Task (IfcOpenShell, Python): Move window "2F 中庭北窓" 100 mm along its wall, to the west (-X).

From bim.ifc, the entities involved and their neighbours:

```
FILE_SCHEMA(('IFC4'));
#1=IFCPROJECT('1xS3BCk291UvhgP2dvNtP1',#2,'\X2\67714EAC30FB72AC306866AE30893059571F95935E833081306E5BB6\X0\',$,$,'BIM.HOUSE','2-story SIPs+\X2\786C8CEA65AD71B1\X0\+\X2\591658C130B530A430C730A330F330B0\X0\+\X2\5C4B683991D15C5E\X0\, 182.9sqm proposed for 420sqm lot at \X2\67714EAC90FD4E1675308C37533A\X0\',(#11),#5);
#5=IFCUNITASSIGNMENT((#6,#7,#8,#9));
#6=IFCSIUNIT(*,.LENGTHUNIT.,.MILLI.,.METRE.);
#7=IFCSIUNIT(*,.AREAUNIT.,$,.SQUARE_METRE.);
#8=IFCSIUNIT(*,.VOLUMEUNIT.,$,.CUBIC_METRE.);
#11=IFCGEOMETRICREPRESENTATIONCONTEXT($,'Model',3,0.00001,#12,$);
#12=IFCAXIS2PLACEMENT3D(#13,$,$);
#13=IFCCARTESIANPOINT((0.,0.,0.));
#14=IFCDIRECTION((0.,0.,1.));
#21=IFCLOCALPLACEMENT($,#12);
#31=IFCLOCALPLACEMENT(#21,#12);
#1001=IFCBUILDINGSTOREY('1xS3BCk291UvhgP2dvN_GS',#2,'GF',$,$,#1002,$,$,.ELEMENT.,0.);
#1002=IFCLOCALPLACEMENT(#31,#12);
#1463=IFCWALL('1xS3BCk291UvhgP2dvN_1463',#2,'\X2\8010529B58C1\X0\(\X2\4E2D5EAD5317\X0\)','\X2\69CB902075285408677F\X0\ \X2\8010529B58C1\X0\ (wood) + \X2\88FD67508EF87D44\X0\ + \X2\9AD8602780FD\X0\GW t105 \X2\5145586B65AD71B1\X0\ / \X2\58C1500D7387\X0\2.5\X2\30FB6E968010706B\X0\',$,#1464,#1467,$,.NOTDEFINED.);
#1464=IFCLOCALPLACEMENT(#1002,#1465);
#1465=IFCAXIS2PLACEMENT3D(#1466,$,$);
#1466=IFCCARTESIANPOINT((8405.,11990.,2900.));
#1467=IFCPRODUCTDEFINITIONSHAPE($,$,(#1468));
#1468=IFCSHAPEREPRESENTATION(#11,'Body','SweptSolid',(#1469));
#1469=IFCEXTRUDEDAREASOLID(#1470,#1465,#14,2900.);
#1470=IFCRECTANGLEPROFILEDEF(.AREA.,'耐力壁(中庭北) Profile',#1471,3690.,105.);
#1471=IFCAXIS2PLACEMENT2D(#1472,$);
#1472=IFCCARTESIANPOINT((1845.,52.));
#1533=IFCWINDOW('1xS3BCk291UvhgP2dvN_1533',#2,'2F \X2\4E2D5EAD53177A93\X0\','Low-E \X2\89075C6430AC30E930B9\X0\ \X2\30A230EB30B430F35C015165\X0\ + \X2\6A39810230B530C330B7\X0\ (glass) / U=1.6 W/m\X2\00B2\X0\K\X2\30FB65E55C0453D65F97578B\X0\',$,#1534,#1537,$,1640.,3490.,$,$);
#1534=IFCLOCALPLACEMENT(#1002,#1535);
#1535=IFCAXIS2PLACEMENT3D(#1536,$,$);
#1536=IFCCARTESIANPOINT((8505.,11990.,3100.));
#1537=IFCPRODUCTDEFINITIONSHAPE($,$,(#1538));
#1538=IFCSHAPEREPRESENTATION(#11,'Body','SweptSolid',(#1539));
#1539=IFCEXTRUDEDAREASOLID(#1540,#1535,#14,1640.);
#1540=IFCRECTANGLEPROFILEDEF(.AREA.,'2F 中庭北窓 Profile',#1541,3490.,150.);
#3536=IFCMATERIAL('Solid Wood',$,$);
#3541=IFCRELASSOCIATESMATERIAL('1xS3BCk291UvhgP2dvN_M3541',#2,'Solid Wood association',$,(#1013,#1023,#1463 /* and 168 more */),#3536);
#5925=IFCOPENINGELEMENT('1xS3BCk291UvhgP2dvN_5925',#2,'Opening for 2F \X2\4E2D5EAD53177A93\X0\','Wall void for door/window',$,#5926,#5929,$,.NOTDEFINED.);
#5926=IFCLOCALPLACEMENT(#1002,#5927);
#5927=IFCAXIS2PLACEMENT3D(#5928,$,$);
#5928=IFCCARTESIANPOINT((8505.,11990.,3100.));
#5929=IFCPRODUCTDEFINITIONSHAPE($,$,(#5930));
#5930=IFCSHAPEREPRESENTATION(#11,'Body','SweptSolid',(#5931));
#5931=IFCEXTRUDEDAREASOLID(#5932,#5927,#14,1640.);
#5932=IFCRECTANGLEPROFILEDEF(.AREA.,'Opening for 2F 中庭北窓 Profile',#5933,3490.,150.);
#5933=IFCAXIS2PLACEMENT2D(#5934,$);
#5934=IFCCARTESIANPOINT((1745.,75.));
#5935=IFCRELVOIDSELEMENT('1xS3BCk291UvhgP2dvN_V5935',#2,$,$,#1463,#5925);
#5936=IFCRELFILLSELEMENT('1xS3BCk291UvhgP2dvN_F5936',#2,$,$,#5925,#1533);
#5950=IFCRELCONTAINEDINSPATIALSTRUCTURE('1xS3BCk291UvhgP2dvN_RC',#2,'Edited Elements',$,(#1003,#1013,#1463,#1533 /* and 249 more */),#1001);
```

```python
import ifcopenshell
import ifcopenshell.api.geometry
import ifcopenshell.util.placement
import ifcopenshell.util.unit

model = ifcopenshell.open("bim.ifc")
unit_scale = ifcopenshell.util.unit.calculate_unit_scale(model)

window = model.by_id(1533)
opening = window.FillsVoids[0].RelatingOpeningElement
wall = opening.VoidsElements[0].RelatingBuildingElement

wall_matrix = ifcopenshell.util.placement.get_local_placement(wall.ObjectPlacement)
shift = wall_matrix[:3, 0] * -0.1 / unit_scale
before = ifcopenshell.util.placement.get_local_placement(window.ObjectPlacement)[:3, 3].copy()

# The window is not placed relative to its opening, so move both.
for product in (opening, window):
    matrix = ifcopenshell.util.placement.get_local_placement(product.ObjectPlacement)
    matrix[:3, 3] += shift
    ifcopenshell.api.geometry.edit_object_placement(model, product=product, matrix=matrix, is_si=False)

after = ifcopenshell.util.placement.get_local_placement(window.ObjectPlacement)[:3, 3]
print("window moved by", (after - before).round(3) + 0.0)

model.write("bim_v2.ifc")
```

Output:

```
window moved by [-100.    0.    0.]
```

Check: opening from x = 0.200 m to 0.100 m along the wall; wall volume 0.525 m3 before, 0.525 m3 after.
